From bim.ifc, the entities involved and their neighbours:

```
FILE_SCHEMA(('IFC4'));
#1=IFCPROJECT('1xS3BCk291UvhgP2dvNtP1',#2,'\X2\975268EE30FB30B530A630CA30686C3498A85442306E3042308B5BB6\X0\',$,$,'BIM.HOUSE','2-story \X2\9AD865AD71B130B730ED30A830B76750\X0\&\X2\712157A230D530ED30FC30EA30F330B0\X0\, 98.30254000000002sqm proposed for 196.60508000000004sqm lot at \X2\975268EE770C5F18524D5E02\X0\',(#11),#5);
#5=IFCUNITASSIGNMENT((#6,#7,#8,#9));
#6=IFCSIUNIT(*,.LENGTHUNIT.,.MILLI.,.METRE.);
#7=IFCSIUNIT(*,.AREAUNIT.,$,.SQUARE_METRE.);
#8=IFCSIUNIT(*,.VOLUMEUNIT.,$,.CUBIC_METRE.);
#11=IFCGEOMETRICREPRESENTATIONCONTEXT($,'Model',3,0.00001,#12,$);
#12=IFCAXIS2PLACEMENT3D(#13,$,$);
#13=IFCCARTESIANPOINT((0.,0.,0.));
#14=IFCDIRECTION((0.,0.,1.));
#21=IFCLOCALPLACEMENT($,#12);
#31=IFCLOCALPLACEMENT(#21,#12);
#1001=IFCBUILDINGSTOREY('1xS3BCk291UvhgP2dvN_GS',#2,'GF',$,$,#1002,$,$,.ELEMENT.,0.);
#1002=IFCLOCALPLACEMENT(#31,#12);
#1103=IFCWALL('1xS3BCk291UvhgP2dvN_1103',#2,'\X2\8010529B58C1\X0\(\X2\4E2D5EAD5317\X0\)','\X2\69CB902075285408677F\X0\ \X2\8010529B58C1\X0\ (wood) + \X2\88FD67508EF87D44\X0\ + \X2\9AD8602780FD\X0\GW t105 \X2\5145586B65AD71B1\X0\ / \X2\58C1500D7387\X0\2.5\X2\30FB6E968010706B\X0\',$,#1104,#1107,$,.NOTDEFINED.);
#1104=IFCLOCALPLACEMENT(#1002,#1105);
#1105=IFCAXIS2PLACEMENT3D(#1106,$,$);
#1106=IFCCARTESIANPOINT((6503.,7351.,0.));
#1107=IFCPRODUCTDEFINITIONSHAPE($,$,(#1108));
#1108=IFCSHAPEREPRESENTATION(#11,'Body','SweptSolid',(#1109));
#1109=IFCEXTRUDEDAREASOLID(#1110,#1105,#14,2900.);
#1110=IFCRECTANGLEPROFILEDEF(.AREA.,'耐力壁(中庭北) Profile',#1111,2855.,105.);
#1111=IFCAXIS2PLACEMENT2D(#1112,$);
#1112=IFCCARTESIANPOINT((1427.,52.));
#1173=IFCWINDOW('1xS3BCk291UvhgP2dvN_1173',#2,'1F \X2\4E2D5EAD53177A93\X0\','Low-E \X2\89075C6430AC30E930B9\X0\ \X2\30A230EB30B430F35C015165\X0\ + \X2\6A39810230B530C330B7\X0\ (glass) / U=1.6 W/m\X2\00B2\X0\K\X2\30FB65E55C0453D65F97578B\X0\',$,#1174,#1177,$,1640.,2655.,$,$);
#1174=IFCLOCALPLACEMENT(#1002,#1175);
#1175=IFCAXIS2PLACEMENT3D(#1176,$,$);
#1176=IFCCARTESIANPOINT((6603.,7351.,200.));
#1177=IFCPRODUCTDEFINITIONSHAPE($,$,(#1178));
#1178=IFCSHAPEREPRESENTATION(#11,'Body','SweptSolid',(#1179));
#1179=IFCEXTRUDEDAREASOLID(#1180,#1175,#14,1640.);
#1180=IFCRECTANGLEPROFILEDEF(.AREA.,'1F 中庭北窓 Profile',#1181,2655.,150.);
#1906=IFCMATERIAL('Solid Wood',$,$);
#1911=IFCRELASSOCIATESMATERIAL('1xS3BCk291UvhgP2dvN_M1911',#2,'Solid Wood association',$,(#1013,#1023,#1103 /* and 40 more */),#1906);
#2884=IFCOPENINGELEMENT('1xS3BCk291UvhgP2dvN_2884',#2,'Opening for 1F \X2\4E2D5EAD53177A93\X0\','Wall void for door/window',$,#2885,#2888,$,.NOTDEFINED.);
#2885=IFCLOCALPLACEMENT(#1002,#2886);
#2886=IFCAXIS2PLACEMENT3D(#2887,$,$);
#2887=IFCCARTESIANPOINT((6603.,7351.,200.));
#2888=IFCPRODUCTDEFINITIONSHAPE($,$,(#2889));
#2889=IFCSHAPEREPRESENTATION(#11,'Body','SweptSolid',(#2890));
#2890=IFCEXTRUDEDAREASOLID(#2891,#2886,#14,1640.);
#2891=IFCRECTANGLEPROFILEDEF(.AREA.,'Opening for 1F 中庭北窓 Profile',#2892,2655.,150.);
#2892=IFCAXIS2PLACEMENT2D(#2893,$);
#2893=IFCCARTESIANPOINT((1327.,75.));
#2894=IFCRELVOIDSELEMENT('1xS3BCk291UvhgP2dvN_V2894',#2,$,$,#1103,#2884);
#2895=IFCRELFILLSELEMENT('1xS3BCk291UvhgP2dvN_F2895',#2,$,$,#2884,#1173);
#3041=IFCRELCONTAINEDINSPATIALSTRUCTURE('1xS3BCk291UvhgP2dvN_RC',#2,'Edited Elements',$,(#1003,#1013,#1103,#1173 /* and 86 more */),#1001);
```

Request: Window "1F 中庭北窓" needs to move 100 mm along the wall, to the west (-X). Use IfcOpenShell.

```python
import ifcopenshell
import ifcopenshell.api.geometry
import ifcopenshell.util.placement
import ifcopenshell.util.unit

model = ifcopenshell.open("bim.ifc")
unit_scale = ifcopenshell.util.unit.calculate_unit_scale(model)

window = model.by_id(1173)
opening = window.FillsVoids[0].RelatingOpeningElement
wall = opening.VoidsElements[0].RelatingBuildingElement

wall_matrix = ifcopenshell.util.placement.get_local_placement(wall.ObjectPlacement)
shift = wall_matrix[:3, 0] * -0.1 / unit_scale
before = ifcopenshell.util.placement.get_local_placement(window.ObjectPlacement)[:3, 3].copy()

# The window is not placed relative to its opening, so move both.
for product in (opening, window):
    matrix = ifcopenshell.util.placement.get_local_placement(product.ObjectPlacement)
    matrix[:3, 3] += shift
    ifcopenshell.api.geometry.edit_object_placement(model, product=product, matrix=matrix, is_si=False)

after = ifcopenshell.util.placement.get_local_placement(window.ObjectPlacement)[:3, 3]
print("window moved by", (after - before).round(3) + 0.0)

model.write("bim-out.ifc")
```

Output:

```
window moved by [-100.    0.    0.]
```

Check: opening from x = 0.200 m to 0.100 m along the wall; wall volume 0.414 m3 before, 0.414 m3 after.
